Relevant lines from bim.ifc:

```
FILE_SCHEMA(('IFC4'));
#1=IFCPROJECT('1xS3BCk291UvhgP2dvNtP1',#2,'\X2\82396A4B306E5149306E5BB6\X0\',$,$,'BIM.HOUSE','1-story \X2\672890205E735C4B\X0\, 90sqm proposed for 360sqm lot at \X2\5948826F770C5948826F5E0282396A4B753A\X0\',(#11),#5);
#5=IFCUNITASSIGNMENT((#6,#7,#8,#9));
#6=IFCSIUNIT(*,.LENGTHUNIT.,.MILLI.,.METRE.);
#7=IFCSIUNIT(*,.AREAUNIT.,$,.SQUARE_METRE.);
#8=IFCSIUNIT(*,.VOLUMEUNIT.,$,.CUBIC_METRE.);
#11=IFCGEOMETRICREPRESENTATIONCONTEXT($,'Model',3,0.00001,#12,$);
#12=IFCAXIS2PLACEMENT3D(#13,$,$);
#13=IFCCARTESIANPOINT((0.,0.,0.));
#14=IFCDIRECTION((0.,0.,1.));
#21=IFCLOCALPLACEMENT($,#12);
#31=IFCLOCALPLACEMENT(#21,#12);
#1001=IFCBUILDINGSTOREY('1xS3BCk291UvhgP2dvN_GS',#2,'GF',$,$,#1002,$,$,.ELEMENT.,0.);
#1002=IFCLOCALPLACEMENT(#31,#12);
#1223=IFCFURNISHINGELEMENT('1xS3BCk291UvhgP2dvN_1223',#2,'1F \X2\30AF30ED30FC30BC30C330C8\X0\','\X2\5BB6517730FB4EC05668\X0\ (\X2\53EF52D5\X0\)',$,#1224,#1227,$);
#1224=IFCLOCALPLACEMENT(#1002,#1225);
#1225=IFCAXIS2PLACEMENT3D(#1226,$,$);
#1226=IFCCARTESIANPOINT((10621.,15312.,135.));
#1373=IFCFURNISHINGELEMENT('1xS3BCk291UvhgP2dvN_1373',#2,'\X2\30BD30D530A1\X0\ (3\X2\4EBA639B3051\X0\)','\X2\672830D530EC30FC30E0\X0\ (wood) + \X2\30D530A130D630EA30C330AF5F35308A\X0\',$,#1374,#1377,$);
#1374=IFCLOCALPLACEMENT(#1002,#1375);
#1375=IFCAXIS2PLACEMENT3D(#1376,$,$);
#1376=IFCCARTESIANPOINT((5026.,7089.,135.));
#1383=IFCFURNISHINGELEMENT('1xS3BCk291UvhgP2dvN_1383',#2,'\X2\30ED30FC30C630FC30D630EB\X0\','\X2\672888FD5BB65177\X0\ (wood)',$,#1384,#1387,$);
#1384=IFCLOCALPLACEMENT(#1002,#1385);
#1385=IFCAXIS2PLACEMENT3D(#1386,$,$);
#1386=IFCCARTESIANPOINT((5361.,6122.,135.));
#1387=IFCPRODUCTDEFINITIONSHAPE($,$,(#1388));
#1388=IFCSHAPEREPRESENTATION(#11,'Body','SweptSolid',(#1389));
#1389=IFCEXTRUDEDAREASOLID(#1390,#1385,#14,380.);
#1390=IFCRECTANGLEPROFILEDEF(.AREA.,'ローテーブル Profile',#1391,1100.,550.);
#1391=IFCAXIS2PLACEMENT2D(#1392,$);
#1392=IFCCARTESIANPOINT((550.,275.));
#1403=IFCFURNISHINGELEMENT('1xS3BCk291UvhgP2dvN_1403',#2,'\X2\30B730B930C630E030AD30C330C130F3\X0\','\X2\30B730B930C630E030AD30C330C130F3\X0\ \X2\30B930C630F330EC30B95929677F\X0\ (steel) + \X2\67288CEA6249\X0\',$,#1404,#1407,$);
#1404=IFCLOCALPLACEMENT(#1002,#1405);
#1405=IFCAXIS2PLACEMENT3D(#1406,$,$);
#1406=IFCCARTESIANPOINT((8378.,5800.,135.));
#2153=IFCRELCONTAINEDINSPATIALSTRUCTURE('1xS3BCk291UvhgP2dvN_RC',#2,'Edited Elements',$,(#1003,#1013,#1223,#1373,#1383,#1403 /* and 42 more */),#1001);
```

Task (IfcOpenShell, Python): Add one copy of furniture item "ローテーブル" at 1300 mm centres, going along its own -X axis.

```python
import ifcopenshell
import ifcopenshell.api.geometry
import ifcopenshell.api.root
import ifcopenshell.util.element
import ifcopenshell.util.placement
import ifcopenshell.util.unit

model = ifcopenshell.open("bim.ifc")
unit_scale = ifcopenshell.util.unit.calculate_unit_scale(model)


def reuse_history(source, copy):
    """copy_class also copies each property set's owner history, people and application; keep the originals."""
    for rel in copy.IsDefinedBy:
        if rel.is_a("IfcRelDefinesByProperties") and (history := rel.RelatingPropertyDefinition.OwnerHistory):
            rel.RelatingPropertyDefinition.OwnerHistory = source.OwnerHistory
            ifcopenshell.util.element.remove_deep2(model, history)


source = model.by_id(1383)
base = ifcopenshell.util.placement.get_local_placement(source.ObjectPlacement)
step = -base[:3, 0] * 1.3 / unit_scale

for i in range(1, 2):
    copy = ifcopenshell.api.root.copy_class(model, product=source)
    copy.Representation = ifcopenshell.util.element.copy_deep(
        model, source.Representation, exclude=["IfcGeometricRepresentationContext", "IfcRepresentationMap"]
    )
    reuse_history(source, copy)
    matrix = base.copy()
    matrix[:3, 3] += i * step
    print("added at", matrix[:3, 3].round(3) + 0.0)
    ifcopenshell.api.geometry.edit_object_placement(model, product=copy, matrix=matrix, is_si=False)

model.write("bim_v2.ifc")
```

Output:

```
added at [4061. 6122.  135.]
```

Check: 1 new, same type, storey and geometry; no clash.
